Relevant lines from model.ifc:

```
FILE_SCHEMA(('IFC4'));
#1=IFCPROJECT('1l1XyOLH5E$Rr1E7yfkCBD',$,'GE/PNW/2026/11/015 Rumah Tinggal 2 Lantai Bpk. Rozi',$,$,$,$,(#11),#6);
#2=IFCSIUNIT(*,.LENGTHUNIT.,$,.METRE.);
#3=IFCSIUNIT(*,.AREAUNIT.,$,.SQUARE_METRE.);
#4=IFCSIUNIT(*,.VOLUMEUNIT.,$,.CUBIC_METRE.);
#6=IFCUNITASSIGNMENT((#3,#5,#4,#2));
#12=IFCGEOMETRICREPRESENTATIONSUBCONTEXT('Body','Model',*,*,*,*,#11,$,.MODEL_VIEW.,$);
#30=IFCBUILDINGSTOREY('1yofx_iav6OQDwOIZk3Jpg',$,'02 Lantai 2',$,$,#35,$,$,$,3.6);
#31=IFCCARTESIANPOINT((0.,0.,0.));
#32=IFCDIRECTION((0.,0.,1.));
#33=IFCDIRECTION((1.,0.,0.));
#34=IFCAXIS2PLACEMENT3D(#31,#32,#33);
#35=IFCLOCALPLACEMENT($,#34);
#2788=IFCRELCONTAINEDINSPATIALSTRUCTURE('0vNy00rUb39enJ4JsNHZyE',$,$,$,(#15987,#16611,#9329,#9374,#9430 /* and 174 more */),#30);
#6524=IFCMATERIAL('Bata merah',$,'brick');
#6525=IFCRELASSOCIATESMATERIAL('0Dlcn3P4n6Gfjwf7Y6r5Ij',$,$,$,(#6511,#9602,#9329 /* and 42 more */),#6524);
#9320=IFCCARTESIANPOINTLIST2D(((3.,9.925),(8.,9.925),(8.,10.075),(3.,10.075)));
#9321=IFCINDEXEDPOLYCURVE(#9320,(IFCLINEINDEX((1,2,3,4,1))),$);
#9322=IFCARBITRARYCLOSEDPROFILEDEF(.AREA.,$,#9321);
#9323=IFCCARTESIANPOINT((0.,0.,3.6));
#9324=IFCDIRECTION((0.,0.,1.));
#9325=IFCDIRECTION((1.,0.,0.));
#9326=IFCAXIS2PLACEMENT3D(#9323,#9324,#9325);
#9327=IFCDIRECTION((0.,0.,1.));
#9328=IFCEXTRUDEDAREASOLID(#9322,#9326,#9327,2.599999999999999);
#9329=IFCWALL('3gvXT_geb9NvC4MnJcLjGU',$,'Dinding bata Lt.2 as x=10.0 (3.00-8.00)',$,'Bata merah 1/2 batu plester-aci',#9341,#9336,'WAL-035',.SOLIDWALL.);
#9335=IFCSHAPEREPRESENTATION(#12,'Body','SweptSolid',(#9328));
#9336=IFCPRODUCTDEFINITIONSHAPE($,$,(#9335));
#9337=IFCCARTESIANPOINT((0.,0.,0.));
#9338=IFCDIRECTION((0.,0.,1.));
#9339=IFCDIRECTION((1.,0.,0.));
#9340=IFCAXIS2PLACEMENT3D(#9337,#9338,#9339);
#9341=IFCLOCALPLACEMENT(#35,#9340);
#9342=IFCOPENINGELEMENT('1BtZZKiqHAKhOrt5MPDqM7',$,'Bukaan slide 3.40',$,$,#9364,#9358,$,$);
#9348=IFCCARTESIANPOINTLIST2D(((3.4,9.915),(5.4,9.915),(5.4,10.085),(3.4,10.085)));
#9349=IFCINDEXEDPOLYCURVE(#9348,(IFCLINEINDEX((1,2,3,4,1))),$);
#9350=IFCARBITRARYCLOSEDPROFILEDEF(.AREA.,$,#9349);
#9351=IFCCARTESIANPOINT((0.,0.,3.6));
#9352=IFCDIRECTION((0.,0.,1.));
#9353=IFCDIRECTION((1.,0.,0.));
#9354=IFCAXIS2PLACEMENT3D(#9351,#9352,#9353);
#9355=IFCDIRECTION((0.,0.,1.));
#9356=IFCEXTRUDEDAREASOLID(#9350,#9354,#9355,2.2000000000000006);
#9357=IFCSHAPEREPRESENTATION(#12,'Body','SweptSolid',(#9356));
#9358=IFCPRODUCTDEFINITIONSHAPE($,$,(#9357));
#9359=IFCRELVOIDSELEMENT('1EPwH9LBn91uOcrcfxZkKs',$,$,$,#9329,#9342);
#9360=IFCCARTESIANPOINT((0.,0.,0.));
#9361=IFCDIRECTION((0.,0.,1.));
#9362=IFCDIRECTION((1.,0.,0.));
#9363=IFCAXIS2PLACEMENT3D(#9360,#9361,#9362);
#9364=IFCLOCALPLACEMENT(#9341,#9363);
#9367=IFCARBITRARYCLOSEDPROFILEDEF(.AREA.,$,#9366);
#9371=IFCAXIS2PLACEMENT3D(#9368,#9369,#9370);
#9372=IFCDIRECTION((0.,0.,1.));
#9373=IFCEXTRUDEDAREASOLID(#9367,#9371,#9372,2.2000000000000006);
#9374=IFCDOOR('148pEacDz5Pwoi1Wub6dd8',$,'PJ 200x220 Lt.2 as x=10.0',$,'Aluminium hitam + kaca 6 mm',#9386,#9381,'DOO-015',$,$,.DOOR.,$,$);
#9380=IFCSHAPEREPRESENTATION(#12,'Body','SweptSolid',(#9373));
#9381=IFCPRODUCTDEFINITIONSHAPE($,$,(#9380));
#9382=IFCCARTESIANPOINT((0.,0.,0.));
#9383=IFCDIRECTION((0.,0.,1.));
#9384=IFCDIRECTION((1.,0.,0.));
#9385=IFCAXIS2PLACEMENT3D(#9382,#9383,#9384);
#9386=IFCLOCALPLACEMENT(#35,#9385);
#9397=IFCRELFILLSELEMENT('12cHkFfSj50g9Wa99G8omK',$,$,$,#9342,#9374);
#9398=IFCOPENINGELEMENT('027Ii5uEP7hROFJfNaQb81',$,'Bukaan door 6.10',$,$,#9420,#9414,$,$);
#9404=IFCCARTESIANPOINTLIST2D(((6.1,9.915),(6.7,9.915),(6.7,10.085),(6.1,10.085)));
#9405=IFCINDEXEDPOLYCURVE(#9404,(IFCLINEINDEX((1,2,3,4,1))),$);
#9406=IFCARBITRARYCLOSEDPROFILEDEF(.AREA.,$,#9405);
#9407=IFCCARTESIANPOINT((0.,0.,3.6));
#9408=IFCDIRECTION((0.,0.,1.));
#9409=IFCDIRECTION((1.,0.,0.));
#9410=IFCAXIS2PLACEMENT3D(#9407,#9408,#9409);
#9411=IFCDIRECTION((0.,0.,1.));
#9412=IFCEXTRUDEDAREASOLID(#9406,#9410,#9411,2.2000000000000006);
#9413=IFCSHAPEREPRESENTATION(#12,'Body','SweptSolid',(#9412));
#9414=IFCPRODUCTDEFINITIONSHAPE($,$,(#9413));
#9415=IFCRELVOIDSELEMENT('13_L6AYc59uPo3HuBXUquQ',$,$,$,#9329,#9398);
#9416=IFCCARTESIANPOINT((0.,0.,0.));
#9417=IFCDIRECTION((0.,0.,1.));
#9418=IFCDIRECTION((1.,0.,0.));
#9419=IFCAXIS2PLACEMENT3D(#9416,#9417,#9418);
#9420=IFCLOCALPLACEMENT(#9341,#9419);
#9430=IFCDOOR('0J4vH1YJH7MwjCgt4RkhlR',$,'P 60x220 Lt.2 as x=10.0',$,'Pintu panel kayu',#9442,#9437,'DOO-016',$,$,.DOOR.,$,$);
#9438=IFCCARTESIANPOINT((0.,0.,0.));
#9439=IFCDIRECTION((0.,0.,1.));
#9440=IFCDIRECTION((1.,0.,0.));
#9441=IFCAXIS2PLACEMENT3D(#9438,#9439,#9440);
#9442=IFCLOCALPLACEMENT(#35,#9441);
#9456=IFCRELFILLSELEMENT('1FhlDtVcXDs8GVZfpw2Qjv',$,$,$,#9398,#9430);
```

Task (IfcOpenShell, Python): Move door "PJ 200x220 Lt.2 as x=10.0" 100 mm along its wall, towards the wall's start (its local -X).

```python
import ifcopenshell
import ifcopenshell.api.geometry
import ifcopenshell.util.placement
import ifcopenshell.util.unit

model = ifcopenshell.open("model.ifc")
unit_scale = ifcopenshell.util.unit.calculate_unit_scale(model)

door = model.by_guid("148pEacDz5Pwoi1Wub6dd8")
opening = door.FillsVoids[0].RelatingOpeningElement
wall = opening.VoidsElements[0].RelatingBuildingElement

wall_matrix = ifcopenshell.util.placement.get_local_placement(wall.ObjectPlacement)
shift = wall_matrix[:3, 0] * -0.1 / unit_scale
before = ifcopenshell.util.placement.get_local_placement(door.ObjectPlacement)[:3, 3].copy()

# The door is not placed relative to its opening, so move both.
for product in (opening, door):
    matrix = ifcopenshell.util.placement.get_local_placement(product.ObjectPlacement)
    matrix[:3, 3] += shift
    ifcopenshell.api.geometry.edit_object_placement(model, product=product, matrix=matrix, is_si=False)

after = ifcopenshell.util.placement.get_local_placement(door.ObjectPlacement)[:3, 3]
print("door moved by", (after - before).round(3) + 0.0)

model.write("model_v2.ifc")
```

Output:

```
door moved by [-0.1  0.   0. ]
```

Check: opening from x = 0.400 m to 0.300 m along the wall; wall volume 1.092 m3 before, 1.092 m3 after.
